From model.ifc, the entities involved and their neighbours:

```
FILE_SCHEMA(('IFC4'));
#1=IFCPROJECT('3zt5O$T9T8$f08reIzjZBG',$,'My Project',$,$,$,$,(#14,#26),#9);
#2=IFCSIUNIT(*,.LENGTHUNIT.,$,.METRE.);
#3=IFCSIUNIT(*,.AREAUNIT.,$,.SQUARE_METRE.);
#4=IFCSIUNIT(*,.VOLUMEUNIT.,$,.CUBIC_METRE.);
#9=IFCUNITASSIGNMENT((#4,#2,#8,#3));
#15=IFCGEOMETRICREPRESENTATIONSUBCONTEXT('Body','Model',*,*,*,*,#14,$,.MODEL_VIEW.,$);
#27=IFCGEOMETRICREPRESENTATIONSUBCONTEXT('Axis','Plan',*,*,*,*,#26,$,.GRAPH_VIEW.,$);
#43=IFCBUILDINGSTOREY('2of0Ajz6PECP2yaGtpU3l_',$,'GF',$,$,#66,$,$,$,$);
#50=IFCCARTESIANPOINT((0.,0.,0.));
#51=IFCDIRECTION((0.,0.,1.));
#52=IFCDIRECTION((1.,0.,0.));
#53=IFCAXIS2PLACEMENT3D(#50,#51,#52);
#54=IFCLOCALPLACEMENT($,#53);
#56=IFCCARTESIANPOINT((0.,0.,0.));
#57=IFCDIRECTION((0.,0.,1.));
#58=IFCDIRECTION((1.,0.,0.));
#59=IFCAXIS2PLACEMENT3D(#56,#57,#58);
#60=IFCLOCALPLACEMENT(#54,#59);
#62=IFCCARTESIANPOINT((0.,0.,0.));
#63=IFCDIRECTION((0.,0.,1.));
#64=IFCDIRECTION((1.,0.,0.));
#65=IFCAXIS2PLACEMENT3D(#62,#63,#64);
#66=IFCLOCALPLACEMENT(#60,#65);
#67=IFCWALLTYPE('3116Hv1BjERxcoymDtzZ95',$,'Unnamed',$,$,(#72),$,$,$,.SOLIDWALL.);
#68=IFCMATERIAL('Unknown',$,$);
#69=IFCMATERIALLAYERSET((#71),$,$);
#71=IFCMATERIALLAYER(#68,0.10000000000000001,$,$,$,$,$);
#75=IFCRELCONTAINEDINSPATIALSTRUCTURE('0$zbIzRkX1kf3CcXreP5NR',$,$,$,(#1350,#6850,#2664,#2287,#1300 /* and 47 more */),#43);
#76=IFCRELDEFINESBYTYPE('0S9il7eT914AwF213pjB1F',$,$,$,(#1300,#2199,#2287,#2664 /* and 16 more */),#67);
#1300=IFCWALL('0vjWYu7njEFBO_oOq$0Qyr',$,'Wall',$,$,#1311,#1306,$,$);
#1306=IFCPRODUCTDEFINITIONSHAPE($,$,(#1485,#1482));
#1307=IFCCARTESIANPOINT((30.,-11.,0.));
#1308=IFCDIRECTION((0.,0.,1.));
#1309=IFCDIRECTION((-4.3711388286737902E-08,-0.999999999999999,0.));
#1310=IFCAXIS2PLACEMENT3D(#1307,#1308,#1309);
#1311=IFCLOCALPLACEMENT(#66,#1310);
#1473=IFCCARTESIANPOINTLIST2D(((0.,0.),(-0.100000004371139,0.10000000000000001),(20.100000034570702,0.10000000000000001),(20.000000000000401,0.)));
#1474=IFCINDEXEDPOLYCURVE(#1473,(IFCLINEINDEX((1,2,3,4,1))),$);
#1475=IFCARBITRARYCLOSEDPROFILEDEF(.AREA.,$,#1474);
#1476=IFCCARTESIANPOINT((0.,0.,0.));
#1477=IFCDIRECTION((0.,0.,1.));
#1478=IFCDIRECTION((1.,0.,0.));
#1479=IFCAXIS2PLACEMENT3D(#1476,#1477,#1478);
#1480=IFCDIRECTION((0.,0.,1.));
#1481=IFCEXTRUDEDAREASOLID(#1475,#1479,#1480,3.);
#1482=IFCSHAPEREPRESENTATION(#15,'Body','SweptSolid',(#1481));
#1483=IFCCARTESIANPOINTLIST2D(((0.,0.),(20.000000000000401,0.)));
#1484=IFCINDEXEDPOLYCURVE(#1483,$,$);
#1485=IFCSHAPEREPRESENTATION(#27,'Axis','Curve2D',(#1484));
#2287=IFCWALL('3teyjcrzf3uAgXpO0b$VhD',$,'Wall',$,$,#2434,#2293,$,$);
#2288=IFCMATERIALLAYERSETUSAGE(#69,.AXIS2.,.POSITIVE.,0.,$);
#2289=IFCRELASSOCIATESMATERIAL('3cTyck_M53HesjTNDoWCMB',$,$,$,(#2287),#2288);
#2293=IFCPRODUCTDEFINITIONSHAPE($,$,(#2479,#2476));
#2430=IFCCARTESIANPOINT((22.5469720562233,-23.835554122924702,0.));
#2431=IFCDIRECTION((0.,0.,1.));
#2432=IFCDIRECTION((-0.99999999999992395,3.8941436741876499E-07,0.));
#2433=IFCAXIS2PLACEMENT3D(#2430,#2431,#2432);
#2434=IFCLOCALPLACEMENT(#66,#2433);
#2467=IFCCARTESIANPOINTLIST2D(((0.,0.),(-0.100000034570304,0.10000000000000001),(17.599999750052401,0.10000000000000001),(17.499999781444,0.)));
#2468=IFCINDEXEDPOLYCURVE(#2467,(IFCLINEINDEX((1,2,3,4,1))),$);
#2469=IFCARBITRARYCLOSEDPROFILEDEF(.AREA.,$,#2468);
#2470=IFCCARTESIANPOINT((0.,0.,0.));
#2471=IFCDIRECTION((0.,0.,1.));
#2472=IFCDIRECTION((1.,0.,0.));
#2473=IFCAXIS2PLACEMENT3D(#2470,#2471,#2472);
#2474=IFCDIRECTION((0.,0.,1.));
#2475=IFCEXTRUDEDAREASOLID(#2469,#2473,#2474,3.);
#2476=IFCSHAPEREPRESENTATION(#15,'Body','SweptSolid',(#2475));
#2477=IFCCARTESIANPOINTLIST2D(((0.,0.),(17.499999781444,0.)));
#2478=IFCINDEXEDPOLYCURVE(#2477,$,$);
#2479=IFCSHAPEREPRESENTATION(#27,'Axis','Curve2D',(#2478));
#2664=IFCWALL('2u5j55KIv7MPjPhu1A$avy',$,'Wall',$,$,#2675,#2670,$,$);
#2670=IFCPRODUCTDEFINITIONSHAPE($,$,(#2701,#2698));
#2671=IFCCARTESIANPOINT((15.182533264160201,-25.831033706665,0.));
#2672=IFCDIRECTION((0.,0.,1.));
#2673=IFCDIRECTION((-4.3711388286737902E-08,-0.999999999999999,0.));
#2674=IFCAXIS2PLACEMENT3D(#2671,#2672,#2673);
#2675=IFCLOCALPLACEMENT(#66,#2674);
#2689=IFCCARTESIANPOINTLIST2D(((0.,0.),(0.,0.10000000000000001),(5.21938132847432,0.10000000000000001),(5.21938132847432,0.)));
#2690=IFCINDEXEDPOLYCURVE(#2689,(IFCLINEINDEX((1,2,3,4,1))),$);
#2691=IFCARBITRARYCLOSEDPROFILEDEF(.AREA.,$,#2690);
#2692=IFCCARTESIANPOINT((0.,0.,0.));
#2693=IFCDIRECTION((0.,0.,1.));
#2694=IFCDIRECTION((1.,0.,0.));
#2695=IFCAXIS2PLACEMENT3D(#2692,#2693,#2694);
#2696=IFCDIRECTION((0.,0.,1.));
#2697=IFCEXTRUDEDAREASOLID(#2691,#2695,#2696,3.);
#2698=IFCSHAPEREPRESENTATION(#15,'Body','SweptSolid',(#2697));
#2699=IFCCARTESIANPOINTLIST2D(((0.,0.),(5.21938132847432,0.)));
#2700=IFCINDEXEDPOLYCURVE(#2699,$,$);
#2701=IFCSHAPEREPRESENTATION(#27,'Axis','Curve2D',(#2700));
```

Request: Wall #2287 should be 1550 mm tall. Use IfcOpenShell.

```python
import ifcopenshell
import ifcopenshell.geom
import ifcopenshell.util.representation
import ifcopenshell.util.shape
import ifcopenshell.util.unit

model = ifcopenshell.open("model.ifc")
unit_scale = ifcopenshell.util.unit.calculate_unit_scale(model)
settings = ifcopenshell.geom.settings()


def volume(element):
    """Net volume in cubic metres, openings subtracted."""
    shape = ifcopenshell.geom.create_shape(settings, element)
    return ifcopenshell.util.shape.get_volume(shape.geometry)


wall = model.by_guid("3teyjcrzf3uAgXpO0b$VhD")
before = volume(wall)

body = ifcopenshell.util.representation.get_representation(wall, "Model", "Body")
solid = body.Items[0]
old_height = solid.Depth
solid.Depth = 1.55 / unit_scale
after = volume(wall)

print(f"height {old_height:g} -> {solid.Depth:g}, volume {before:.3f} -> {after:.3f} m3")

model.write("model_rev.ifc")
```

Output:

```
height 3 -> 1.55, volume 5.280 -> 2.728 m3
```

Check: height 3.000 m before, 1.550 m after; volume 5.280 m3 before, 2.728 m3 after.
